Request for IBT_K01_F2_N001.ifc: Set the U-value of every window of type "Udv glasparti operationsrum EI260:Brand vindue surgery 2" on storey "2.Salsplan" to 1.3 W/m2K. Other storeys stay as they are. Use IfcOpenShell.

First a look at what the model holds.

```python
import ifcopenshell
import ifcopenshell.util.element

model = ifcopenshell.open("IBT_K01_F2_N001.ifc")
print(model.schema)
storey = next(s for s in model.by_type("IfcBuildingStorey") if s.Name == "2.Salsplan")
windows = [e for e in ifcopenshell.util.element.get_decomposition(storey) if e.is_a("IfcWindow")]
seen = {}
for e in windows:
    element_type = ifcopenshell.util.element.get_type(e)
    key = (element_type.Name if element_type != e and element_type else None, ifcopenshell.util.element.get_pset(e, "Pset_WindowCommon", "ThermalTransmittance"))
    seen[key] = seen.get(key, 0) + 1
for (name, value), count in sorted(seen.items(), key=str):
    print(count, "x", name, "|", value)
```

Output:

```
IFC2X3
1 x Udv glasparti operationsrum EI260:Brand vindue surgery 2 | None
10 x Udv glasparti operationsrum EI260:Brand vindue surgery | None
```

```python
import ifcopenshell
import ifcopenshell.api.pset
import ifcopenshell.util.element

model = ifcopenshell.open("IBT_K01_F2_N001.ifc")

storey = next(s for s in model.by_type("IfcBuildingStorey") if s.Name == "2.Salsplan")
windows = [e for e in ifcopenshell.util.element.get_decomposition(storey) if e.is_a("IfcWindow")]

count = 0
for e in windows:
    element_type = ifcopenshell.util.element.get_type(e)
    if element_type in (None, e) or element_type.Name != "Udv glasparti operationsrum EI260:Brand vindue surgery 2":
        continue
    # add_pset returns the element's existing set when there is one.
    pset = ifcopenshell.api.pset.add_pset(model, product=e, name="Pset_WindowCommon")
    ifcopenshell.api.pset.edit_pset(model, pset=pset, properties={"ThermalTransmittance": 1.3})
    count += 1

print(count, "windows updated")

model.write("IBT_K01_F2_N001-out.ifc")
```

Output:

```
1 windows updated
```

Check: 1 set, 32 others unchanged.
